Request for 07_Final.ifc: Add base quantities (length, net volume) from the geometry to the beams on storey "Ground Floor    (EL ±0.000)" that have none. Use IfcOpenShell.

First a look at what the model holds.

```python
import ifcopenshell
import ifcopenshell.util.element
import ifcopenshell.util.unit

model = ifcopenshell.open("07_Final.ifc")
print(model.schema)
for unit_type in ("LENGTHUNIT", "AREAUNIT", "VOLUMEUNIT"):
    print(unit_type, ifcopenshell.util.unit.calculate_unit_scale(model, unit_type))
storey = next(s for s in model.by_type("IfcBuildingStorey") if s.Name == "Ground Floor    (EL ±0.000)")
beams = [e for e in ifcopenshell.util.element.get_decomposition(storey) if e.is_a("IfcBeam")]
for e in sorted(beams, key=lambda e: e.id()):
    print(e.id(), e.is_a(), e.Name, list(ifcopenshell.util.element.get_psets(e, qtos_only=True)), sep=" | ")
```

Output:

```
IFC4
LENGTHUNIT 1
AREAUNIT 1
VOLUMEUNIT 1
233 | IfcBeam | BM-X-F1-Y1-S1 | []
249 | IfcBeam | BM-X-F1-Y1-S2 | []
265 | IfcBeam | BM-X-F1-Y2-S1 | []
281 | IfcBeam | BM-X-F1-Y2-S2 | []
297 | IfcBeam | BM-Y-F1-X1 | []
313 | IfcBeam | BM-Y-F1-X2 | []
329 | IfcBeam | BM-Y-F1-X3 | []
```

```python
import ifcopenshell
import ifcopenshell.api.pset
import ifcopenshell.geom
import ifcopenshell.util.element
import ifcopenshell.util.shape
import ifcopenshell.util.unit

model = ifcopenshell.open("07_Final.ifc")
unit_scale = ifcopenshell.util.unit.calculate_unit_scale(model)
volume_scale = ifcopenshell.util.unit.calculate_unit_scale(model, "VOLUMEUNIT")
settings = ifcopenshell.geom.settings()

storey = next(s for s in model.by_type("IfcBuildingStorey") if s.Name == "Ground Floor    (EL ±0.000)")
beams = [e for e in ifcopenshell.util.element.get_decomposition(storey) if e.is_a("IfcBeam")]

for e in sorted(beams, key=lambda e: e.id()):
    if ifcopenshell.util.element.get_psets(e, qtos_only=True, should_inherit=False):
        continue
    # Geometry comes back in metres, in the element's own axes.
    shape = ifcopenshell.geom.create_shape(settings, e)
    values = {
        "Length": ifcopenshell.util.shape.get_max_xyz(shape.geometry) / unit_scale,
        "NetVolume": ifcopenshell.util.shape.get_volume(shape.geometry) / volume_scale,
    }
    qto = ifcopenshell.api.pset.add_qto(model, product=e, name="Qto_BeamBaseQuantities")
    ifcopenshell.api.pset.edit_qto(model, qto=qto, properties=values)
    print(e.id(), {k: round(v, 3) for k, v in values.items()})

model.write("07_Final_edited.ifc")
```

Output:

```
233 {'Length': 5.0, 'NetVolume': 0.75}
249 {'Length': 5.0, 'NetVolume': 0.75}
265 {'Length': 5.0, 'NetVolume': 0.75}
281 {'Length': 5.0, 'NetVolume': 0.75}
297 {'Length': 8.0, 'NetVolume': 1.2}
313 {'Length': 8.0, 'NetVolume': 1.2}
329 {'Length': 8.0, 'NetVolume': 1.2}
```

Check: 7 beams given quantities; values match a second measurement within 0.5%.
